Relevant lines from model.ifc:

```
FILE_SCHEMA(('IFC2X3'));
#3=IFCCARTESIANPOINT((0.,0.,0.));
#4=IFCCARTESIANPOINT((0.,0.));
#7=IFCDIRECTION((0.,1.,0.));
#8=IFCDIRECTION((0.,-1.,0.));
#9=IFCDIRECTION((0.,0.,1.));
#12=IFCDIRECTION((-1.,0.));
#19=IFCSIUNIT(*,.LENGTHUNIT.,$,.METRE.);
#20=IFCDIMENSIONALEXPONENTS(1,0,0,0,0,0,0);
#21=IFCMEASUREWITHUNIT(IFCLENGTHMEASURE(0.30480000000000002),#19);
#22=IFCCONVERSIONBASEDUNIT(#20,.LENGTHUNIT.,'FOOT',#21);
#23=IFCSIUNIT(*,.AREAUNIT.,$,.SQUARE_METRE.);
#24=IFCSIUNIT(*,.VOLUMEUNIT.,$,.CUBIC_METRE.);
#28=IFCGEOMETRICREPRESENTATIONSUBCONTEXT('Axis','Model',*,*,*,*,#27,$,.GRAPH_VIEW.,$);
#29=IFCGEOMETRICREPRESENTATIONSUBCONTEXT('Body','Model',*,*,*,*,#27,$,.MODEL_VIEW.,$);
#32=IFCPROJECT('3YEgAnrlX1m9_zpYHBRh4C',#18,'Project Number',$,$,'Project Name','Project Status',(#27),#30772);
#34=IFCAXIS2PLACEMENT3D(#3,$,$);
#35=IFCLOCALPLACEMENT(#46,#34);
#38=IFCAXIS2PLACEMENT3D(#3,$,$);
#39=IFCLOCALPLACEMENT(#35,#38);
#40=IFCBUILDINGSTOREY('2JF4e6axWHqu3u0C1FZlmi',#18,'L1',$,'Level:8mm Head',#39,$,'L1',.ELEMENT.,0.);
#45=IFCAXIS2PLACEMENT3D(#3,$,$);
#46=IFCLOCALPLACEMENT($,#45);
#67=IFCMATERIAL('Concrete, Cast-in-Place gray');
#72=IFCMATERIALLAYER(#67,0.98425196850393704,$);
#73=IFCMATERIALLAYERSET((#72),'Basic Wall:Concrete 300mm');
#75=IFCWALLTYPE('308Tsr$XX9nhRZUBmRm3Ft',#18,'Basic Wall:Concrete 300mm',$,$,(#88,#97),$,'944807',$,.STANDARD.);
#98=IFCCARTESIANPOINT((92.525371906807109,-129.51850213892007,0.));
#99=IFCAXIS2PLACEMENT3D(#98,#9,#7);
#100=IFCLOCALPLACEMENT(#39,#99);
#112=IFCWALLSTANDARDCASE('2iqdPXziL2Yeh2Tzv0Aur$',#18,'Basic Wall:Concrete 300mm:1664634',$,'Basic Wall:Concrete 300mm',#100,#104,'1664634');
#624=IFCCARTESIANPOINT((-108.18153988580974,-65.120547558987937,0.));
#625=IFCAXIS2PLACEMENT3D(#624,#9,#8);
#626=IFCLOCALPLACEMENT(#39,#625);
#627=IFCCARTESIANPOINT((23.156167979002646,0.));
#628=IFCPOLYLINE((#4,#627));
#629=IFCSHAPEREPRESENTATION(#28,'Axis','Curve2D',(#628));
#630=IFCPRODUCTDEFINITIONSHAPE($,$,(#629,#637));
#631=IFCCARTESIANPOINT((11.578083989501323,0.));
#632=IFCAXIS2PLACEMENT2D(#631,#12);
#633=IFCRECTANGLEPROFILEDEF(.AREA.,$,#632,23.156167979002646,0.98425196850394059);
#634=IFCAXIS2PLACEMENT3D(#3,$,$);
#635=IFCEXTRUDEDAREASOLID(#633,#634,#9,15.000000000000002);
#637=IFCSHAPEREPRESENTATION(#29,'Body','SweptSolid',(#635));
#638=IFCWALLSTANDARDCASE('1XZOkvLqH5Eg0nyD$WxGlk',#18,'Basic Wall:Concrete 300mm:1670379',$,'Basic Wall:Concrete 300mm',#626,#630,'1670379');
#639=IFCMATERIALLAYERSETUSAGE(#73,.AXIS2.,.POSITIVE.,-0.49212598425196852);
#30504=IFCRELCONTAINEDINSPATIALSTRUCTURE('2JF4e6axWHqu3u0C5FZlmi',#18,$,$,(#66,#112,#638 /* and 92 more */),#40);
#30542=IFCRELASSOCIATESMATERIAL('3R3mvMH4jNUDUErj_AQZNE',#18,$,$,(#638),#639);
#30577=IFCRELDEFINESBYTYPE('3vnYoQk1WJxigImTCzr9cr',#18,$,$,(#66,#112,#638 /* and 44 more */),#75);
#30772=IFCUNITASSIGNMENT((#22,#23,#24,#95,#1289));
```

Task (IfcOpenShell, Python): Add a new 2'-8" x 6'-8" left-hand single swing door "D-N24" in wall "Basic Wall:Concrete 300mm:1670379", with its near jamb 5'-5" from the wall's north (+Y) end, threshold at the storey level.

```python
import numpy as np
import ifcopenshell
import ifcopenshell.api.feature
import ifcopenshell.api.geometry
import ifcopenshell.api.root
import ifcopenshell.api.spatial
import ifcopenshell.api.type
import ifcopenshell.geom
import ifcopenshell.util.element
import ifcopenshell.util.placement
import ifcopenshell.util.representation
import ifcopenshell.util.shape
import ifcopenshell.util.unit

model = ifcopenshell.open("model.ifc")
unit_scale = ifcopenshell.util.unit.calculate_unit_scale(model)
settings = ifcopenshell.geom.settings()


def volume(element):
    """Net volume in cubic metres, openings subtracted."""
    shape = ifcopenshell.geom.create_shape(settings, element)
    return ifcopenshell.util.shape.get_volume(shape.geometry)


wall = model.by_guid("1XZOkvLqH5Eg0nyD$WxGlk")
storey = ifcopenshell.util.element.get_container(wall, ifc_class="IfcBuildingStorey")
context = ifcopenshell.util.representation.get_context(model, "Model", "Body", "MODEL_VIEW")
before = volume(wall)

width, height, from_end, sill = 0.8128, 2.032, 1.651, 0.0  # metres

# The wall runs along its own X axis, and the end named is its -X end.
wall_shape = ifcopenshell.geom.create_shape(settings, wall)
x, y, z = ifcopenshell.util.shape.get_vertices(wall_shape.geometry).T
start = x.min() + from_end
face, thickness = float(y.min()), float(y.max() - y.min())
wall_matrix = ifcopenshell.util.placement.get_local_placement(wall.ObjectPlacement)
level = ifcopenshell.util.placement.get_local_placement(storey.ObjectPlacement)[2, 3]


def in_wall(x, y):
    """Placement at x, y metres in the wall's axes, at sill height."""
    matrix = wall_matrix.copy()
    matrix[:, 3] = wall_matrix @ np.array([x / unit_scale, y / unit_scale, 0.0, 1.0])
    matrix[2, 3] = level + sill / unit_scale
    return matrix


# Opening: a box that overshoots both wall faces by 50 mm.
opening = ifcopenshell.api.root.create_entity(model, ifc_class="IfcOpeningElement")
box = ifcopenshell.api.geometry.add_wall_representation(
    model, context=context, length=width, height=height, thickness=thickness + 0.1
)
ifcopenshell.api.geometry.assign_representation(model, product=opening, representation=box)
ifcopenshell.api.geometry.edit_object_placement(model, product=opening, matrix=in_wall(start, face - 0.05), is_si=False)
ifcopenshell.api.feature.add_feature(model, feature=opening, element=wall)

door = ifcopenshell.api.root.create_entity(model, ifc_class="IfcDoor", name="D-N24")
door.OverallWidth, door.OverallHeight = width / unit_scale, height / unit_scale
body = ifcopenshell.api.geometry.add_door_representation(
    model,
    context=context,
    overall_width=door.OverallWidth,
    overall_height=door.OverallHeight,
    operation_type="SINGLE_SWING_LEFT",
    lining_properties={"LiningDepth": thickness / unit_scale, "ThresholdDepth": thickness / unit_scale},
)
ifcopenshell.api.geometry.assign_representation(model, product=door, representation=body)
ifcopenshell.api.spatial.assign_container(model, products=[door], relating_structure=storey)
fills = ifcopenshell.api.feature.add_filling(model, opening=opening, element=door)
fills.OwnerHistory = door.OwnerHistory  # required in IFC2X3

# IFC2X3 keeps the operation on the door style.
style = ifcopenshell.api.root.create_entity(model, ifc_class="IfcDoorStyle", name="D-N24")
style.OperationType, style.ConstructionType = "SINGLE_SWING_LEFT", "NOTDEFINED"
style.ParameterTakesPrecedence = style.Sizeable = False
ifcopenshell.api.type.assign_type(model, related_objects=[door], relating_type=style)

# The lining spans the wall, so the door starts at the wall face.
ifcopenshell.api.geometry.edit_object_placement(model, product=door, matrix=in_wall(start, face), is_si=False)

after = volume(wall)

print(f"wall volume {before:.3f} -> {after:.3f} m3")

model.write("model_edited.ifc")
```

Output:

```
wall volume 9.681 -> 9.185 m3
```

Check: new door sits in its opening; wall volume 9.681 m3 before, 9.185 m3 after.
